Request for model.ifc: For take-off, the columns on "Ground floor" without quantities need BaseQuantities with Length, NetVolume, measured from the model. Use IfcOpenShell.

First a look at what the model holds.

```python
import ifcopenshell
import ifcopenshell.util.element
import ifcopenshell.util.unit

model = ifcopenshell.open("model.ifc")
print(model.schema)
for unit_type in ("LENGTHUNIT", "AREAUNIT", "VOLUMEUNIT"):
    print(unit_type, ifcopenshell.util.unit.calculate_unit_scale(model, unit_type))
storey = next(s for s in model.by_type("IfcBuildingStorey") if s.Name == "Ground floor")
columns = [e for e in ifcopenshell.util.element.get_decomposition(storey) if e.is_a("IfcColumn")]
for e in sorted(columns, key=lambda e: e.id()):
    print(e.id(), e.is_a(), e.Name, list(ifcopenshell.util.element.get_psets(e, qtos_only=True)), sep=" | ")
```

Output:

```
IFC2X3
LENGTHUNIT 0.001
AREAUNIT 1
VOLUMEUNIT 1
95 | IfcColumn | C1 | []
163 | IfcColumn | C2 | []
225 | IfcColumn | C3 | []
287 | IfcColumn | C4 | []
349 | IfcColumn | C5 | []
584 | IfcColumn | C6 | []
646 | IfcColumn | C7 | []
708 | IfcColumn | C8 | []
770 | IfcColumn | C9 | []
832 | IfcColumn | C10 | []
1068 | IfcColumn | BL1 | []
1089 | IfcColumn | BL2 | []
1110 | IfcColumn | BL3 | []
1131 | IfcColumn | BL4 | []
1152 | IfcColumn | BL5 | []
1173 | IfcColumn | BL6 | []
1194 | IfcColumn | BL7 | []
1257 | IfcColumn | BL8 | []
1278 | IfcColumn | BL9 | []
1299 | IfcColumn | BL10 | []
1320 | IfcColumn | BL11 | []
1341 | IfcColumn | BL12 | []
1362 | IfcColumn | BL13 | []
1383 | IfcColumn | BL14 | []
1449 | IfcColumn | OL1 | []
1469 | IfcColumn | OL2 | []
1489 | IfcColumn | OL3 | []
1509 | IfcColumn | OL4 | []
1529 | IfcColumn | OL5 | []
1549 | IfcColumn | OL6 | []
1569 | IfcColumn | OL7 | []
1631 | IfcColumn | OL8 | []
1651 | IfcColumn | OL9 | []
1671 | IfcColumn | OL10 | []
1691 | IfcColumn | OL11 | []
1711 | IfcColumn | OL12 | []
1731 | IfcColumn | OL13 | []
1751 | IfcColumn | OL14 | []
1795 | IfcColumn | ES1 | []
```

```python
import ifcopenshell
import ifcopenshell.api.pset
import ifcopenshell.geom
import ifcopenshell.util.element
import ifcopenshell.util.shape
import ifcopenshell.util.unit

model = ifcopenshell.open("model.ifc")
unit_scale = ifcopenshell.util.unit.calculate_unit_scale(model)
volume_scale = ifcopenshell.util.unit.calculate_unit_scale(model, "VOLUMEUNIT")
settings = ifcopenshell.geom.settings()

storey = next(s for s in model.by_type("IfcBuildingStorey") if s.Name == "Ground floor")
columns = [e for e in ifcopenshell.util.element.get_decomposition(storey) if e.is_a("IfcColumn")]

for e in sorted(columns, key=lambda e: e.id()):
    if ifcopenshell.util.element.get_psets(e, qtos_only=True, should_inherit=False):
        continue
    # Geometry comes back in metres, in the element's own axes.
    shape = ifcopenshell.geom.create_shape(settings, e)
    values = {
        "Length": ifcopenshell.util.shape.get_z(shape.geometry) / unit_scale,
        "NetVolume": ifcopenshell.util.shape.get_volume(shape.geometry) / volume_scale,
    }
    qto = ifcopenshell.api.pset.add_qto(model, product=e, name="BaseQuantities")
    ifcopenshell.api.pset.edit_qto(model, qto=qto, properties=values)
    print(e.id(), {k: round(v, 3) for k, v in values.items()})

model.write("model_edited.ifc")
```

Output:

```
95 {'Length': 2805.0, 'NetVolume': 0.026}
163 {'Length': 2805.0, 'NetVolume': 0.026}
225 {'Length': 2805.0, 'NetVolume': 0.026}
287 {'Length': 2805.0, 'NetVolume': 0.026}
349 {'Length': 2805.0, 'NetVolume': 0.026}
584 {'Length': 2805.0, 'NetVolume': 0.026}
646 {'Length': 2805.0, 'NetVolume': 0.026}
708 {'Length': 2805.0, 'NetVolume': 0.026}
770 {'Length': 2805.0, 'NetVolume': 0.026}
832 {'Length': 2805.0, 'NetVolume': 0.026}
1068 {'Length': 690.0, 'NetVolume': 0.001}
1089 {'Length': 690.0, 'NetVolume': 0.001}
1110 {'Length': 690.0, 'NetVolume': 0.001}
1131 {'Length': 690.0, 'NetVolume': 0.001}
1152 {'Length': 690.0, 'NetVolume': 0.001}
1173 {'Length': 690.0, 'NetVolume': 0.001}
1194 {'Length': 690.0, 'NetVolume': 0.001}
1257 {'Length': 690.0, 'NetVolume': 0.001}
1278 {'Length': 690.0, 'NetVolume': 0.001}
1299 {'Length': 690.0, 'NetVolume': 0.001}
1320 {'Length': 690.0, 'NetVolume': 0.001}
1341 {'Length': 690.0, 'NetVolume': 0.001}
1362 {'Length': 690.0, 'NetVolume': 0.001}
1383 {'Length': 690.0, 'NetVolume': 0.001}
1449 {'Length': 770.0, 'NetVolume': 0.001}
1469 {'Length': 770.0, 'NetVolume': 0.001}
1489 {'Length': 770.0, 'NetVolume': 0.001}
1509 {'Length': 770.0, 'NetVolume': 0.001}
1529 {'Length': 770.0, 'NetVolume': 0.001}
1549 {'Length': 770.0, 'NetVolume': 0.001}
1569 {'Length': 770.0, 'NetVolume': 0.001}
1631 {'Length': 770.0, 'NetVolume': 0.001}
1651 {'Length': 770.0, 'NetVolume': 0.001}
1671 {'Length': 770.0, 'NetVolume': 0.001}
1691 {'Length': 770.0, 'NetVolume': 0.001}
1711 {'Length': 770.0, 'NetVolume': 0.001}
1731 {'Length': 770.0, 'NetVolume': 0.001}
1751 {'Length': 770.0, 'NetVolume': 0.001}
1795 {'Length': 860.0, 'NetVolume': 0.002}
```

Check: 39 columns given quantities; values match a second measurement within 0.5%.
